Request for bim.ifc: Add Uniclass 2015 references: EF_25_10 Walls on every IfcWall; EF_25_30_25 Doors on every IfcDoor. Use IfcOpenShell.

First a look at what the model holds.

```python
import ifcopenshell

model = ifcopenshell.open("bim.ifc")
print(model.schema)
print("classifications:", [c.Name for c in model.by_type("IfcClassification")])
for ifc_class in ("IfcDoor", "IfcRoof", "IfcStair", "IfcWall", "IfcWindow"):
    print(ifc_class, len(model.by_type(ifc_class)))
```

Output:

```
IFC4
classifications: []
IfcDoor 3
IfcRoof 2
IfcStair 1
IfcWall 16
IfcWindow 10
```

```python
import ifcopenshell
import ifcopenshell.api.classification

model = ifcopenshell.open("bim.ifc")

system = ifcopenshell.api.classification.add_classification(model, classification="Uniclass 2015")

codes = {
    "IfcWall": ("EF_25_10", "Walls"),
    "IfcDoor": ("EF_25_30_25", "Doors"),
}
for ifc_class, (code, name) in codes.items():
    products = model.by_type(ifc_class)
    ifcopenshell.api.classification.add_reference(
        model, products=products, classification=system, identification=code, name=name
    )
    print(code, len(products))

model.write("bim_updated.ifc")
```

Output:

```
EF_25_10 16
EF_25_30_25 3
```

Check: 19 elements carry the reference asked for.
